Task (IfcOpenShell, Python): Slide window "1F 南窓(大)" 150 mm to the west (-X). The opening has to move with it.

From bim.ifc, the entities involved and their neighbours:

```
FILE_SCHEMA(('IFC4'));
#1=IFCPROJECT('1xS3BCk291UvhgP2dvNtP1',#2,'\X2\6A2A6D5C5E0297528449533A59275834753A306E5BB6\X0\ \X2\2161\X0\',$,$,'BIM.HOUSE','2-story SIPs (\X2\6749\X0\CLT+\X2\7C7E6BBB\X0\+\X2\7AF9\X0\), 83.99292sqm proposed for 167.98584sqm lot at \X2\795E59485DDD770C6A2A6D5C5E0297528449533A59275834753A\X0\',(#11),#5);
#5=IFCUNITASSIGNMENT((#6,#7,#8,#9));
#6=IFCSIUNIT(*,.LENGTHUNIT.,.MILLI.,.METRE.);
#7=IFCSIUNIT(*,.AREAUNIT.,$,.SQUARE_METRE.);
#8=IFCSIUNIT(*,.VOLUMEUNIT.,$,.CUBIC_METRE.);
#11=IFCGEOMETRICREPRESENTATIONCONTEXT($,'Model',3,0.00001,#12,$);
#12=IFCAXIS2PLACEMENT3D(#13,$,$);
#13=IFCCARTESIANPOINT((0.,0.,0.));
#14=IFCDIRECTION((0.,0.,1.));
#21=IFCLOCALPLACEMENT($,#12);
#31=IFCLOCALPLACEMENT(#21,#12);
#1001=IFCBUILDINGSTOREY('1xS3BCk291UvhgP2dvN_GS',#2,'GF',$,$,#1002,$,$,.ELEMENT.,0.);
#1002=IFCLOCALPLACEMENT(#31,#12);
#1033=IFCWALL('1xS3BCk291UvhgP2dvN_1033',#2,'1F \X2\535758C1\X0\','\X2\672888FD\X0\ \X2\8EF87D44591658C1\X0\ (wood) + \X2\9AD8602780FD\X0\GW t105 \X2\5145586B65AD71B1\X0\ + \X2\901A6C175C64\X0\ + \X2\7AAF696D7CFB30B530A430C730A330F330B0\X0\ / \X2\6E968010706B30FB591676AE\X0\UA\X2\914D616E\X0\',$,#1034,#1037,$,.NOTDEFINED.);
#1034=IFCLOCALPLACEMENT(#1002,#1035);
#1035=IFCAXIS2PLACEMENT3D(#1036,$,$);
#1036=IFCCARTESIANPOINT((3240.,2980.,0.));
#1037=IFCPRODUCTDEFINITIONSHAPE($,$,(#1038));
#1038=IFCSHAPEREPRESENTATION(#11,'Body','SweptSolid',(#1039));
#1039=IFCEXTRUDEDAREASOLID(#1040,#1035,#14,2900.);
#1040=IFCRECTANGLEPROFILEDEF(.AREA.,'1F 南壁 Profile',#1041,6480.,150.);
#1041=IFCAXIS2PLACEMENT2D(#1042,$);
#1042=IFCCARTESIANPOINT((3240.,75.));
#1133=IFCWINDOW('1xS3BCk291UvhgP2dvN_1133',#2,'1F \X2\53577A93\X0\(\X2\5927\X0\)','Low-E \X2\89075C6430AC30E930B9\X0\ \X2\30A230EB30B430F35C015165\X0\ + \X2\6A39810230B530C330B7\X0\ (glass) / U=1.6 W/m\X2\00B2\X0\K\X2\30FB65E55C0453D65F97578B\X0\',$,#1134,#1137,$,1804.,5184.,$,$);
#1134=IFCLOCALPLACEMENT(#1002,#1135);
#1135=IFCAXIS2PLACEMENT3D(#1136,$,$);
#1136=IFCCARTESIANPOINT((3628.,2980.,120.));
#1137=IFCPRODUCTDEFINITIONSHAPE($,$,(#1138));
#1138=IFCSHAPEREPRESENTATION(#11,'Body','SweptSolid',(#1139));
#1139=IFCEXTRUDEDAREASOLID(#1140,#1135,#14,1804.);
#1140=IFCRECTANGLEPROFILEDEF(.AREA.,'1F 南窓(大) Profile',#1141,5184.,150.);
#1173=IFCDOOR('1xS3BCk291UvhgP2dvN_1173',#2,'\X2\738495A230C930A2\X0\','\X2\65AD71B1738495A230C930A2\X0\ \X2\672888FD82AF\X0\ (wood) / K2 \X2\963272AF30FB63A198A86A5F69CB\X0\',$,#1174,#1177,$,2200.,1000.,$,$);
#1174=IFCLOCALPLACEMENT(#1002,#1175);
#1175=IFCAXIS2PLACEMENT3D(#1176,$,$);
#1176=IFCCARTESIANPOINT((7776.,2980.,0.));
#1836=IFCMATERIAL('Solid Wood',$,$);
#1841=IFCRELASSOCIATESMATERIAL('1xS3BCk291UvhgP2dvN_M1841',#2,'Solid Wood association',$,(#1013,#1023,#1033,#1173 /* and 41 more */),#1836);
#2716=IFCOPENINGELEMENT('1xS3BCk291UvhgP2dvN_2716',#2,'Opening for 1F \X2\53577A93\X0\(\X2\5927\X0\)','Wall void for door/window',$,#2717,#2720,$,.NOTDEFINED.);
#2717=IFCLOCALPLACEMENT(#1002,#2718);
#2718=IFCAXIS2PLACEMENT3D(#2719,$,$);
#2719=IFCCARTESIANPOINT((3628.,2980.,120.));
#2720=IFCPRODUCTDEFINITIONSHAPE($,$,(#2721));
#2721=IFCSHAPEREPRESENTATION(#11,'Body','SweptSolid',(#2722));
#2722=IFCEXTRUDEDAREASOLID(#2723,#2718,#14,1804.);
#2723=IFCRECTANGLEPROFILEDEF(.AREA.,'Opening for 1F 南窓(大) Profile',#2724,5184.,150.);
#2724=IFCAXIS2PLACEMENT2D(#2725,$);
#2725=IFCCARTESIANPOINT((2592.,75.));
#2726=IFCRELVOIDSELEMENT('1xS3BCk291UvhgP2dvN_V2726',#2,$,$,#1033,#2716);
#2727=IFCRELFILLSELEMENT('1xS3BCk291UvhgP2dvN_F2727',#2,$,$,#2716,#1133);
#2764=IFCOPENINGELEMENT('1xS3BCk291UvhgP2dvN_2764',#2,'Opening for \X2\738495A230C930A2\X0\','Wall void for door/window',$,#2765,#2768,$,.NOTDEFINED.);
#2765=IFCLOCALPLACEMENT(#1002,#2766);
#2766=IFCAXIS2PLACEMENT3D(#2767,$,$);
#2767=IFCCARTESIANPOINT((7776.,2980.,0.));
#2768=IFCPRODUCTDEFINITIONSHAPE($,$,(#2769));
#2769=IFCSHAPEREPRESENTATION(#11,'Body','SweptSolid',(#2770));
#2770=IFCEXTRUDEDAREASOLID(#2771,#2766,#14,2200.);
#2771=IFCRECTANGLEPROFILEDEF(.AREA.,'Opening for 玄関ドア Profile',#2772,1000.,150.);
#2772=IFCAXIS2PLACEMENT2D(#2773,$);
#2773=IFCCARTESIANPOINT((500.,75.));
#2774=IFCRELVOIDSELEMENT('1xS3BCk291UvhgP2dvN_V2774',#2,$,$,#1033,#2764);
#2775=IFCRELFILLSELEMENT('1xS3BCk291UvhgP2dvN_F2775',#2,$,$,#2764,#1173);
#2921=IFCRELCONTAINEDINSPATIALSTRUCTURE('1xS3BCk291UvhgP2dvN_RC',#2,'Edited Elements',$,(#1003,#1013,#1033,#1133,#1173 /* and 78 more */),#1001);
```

```python
import ifcopenshell
import ifcopenshell.api.geometry
import ifcopenshell.util.placement

model = ifcopenshell.open("bim.ifc")

window = model.by_id(1133)
opening = window.FillsVoids[0].RelatingOpeningElement
wall = opening.VoidsElements[0].RelatingBuildingElement

wall_matrix = ifcopenshell.util.placement.get_local_placement(wall.ObjectPlacement)
shift = wall_matrix[:3, 0] * -150.0
before = ifcopenshell.util.placement.get_local_placement(window.ObjectPlacement)[:3, 3].copy()

# The window is not placed relative to its opening, so move both.
for product in (opening, window):
    matrix = ifcopenshell.util.placement.get_local_placement(product.ObjectPlacement)
    matrix[:3, 3] += shift
    ifcopenshell.api.geometry.edit_object_placement(model, product=product, matrix=matrix, is_si=False)

after = ifcopenshell.util.placement.get_local_placement(window.ObjectPlacement)[:3, 3]
print("window moved by", (after - before).round(3) + 0.0)

model.write("bim_rev.ifc")
```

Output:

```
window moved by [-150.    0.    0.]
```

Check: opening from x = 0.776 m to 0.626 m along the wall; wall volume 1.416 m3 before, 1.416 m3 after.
